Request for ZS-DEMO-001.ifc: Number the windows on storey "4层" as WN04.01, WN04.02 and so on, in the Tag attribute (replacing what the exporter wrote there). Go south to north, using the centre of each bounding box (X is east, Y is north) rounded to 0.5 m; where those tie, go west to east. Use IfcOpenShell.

First a look at what the model holds.

```python
import ifcopenshell
import ifcopenshell.util.element
import ifcopenshell.util.placement

model = ifcopenshell.open("ZS-DEMO-001.ifc")
print(model.schema)
storey = next(s for s in model.by_type("IfcBuildingStorey") if s.Name == "4层")
windows = [e for e in ifcopenshell.util.element.get_decomposition(storey) if e.is_a("IfcWindow")]
for e in sorted(windows, key=lambda e: e.id()):
    origin = ifcopenshell.util.placement.get_local_placement(e.ObjectPlacement)[:3, 3]
    print(e.id(), e.Tag, e.Name, origin.round(2) + 0.0, sep=" | ")
```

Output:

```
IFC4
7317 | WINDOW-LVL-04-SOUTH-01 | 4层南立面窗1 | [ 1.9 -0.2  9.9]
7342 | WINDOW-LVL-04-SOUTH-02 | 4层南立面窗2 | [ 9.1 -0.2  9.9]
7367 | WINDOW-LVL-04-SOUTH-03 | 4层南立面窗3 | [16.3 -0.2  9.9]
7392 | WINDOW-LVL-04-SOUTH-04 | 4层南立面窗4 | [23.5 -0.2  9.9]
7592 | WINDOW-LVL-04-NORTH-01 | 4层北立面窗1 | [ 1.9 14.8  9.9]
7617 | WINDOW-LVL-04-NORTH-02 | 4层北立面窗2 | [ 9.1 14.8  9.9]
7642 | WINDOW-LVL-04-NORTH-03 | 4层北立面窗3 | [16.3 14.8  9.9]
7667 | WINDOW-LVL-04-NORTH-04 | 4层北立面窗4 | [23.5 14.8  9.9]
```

```python
import ifcopenshell
import ifcopenshell.geom
import ifcopenshell.util.element
import ifcopenshell.util.shape

model = ifcopenshell.open("ZS-DEMO-001.ifc")
settings = ifcopenshell.geom.settings()
settings.set("use-world-coords", True)


def centre(element):
    shape = ifcopenshell.geom.create_shape(settings, element)
    return ifcopenshell.util.shape.get_bbox_centroid(shape.geometry)


storey = next(s for s in model.by_type("IfcBuildingStorey") if s.Name == "4层")
windows = [e for e in ifcopenshell.util.element.get_decomposition(storey) if e.is_a("IfcWindow")]

# Insertion points can sit at a corner or the storey origin, so sort by the geometry (in metres).
centres = {e: centre(e) for e in windows}
windows.sort(key=lambda e: (round(centres[e][1] / 0.5), centres[e][0]))

for i, e in enumerate(windows, start=1):
    number = f"WN04.{i:02d}"
    e.Tag = number
    print(e.id(), number)

model.write("ZS-DEMO-001_updated.ifc")
```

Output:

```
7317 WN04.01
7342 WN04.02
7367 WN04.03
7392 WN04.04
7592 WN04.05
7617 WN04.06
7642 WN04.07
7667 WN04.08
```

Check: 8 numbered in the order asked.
